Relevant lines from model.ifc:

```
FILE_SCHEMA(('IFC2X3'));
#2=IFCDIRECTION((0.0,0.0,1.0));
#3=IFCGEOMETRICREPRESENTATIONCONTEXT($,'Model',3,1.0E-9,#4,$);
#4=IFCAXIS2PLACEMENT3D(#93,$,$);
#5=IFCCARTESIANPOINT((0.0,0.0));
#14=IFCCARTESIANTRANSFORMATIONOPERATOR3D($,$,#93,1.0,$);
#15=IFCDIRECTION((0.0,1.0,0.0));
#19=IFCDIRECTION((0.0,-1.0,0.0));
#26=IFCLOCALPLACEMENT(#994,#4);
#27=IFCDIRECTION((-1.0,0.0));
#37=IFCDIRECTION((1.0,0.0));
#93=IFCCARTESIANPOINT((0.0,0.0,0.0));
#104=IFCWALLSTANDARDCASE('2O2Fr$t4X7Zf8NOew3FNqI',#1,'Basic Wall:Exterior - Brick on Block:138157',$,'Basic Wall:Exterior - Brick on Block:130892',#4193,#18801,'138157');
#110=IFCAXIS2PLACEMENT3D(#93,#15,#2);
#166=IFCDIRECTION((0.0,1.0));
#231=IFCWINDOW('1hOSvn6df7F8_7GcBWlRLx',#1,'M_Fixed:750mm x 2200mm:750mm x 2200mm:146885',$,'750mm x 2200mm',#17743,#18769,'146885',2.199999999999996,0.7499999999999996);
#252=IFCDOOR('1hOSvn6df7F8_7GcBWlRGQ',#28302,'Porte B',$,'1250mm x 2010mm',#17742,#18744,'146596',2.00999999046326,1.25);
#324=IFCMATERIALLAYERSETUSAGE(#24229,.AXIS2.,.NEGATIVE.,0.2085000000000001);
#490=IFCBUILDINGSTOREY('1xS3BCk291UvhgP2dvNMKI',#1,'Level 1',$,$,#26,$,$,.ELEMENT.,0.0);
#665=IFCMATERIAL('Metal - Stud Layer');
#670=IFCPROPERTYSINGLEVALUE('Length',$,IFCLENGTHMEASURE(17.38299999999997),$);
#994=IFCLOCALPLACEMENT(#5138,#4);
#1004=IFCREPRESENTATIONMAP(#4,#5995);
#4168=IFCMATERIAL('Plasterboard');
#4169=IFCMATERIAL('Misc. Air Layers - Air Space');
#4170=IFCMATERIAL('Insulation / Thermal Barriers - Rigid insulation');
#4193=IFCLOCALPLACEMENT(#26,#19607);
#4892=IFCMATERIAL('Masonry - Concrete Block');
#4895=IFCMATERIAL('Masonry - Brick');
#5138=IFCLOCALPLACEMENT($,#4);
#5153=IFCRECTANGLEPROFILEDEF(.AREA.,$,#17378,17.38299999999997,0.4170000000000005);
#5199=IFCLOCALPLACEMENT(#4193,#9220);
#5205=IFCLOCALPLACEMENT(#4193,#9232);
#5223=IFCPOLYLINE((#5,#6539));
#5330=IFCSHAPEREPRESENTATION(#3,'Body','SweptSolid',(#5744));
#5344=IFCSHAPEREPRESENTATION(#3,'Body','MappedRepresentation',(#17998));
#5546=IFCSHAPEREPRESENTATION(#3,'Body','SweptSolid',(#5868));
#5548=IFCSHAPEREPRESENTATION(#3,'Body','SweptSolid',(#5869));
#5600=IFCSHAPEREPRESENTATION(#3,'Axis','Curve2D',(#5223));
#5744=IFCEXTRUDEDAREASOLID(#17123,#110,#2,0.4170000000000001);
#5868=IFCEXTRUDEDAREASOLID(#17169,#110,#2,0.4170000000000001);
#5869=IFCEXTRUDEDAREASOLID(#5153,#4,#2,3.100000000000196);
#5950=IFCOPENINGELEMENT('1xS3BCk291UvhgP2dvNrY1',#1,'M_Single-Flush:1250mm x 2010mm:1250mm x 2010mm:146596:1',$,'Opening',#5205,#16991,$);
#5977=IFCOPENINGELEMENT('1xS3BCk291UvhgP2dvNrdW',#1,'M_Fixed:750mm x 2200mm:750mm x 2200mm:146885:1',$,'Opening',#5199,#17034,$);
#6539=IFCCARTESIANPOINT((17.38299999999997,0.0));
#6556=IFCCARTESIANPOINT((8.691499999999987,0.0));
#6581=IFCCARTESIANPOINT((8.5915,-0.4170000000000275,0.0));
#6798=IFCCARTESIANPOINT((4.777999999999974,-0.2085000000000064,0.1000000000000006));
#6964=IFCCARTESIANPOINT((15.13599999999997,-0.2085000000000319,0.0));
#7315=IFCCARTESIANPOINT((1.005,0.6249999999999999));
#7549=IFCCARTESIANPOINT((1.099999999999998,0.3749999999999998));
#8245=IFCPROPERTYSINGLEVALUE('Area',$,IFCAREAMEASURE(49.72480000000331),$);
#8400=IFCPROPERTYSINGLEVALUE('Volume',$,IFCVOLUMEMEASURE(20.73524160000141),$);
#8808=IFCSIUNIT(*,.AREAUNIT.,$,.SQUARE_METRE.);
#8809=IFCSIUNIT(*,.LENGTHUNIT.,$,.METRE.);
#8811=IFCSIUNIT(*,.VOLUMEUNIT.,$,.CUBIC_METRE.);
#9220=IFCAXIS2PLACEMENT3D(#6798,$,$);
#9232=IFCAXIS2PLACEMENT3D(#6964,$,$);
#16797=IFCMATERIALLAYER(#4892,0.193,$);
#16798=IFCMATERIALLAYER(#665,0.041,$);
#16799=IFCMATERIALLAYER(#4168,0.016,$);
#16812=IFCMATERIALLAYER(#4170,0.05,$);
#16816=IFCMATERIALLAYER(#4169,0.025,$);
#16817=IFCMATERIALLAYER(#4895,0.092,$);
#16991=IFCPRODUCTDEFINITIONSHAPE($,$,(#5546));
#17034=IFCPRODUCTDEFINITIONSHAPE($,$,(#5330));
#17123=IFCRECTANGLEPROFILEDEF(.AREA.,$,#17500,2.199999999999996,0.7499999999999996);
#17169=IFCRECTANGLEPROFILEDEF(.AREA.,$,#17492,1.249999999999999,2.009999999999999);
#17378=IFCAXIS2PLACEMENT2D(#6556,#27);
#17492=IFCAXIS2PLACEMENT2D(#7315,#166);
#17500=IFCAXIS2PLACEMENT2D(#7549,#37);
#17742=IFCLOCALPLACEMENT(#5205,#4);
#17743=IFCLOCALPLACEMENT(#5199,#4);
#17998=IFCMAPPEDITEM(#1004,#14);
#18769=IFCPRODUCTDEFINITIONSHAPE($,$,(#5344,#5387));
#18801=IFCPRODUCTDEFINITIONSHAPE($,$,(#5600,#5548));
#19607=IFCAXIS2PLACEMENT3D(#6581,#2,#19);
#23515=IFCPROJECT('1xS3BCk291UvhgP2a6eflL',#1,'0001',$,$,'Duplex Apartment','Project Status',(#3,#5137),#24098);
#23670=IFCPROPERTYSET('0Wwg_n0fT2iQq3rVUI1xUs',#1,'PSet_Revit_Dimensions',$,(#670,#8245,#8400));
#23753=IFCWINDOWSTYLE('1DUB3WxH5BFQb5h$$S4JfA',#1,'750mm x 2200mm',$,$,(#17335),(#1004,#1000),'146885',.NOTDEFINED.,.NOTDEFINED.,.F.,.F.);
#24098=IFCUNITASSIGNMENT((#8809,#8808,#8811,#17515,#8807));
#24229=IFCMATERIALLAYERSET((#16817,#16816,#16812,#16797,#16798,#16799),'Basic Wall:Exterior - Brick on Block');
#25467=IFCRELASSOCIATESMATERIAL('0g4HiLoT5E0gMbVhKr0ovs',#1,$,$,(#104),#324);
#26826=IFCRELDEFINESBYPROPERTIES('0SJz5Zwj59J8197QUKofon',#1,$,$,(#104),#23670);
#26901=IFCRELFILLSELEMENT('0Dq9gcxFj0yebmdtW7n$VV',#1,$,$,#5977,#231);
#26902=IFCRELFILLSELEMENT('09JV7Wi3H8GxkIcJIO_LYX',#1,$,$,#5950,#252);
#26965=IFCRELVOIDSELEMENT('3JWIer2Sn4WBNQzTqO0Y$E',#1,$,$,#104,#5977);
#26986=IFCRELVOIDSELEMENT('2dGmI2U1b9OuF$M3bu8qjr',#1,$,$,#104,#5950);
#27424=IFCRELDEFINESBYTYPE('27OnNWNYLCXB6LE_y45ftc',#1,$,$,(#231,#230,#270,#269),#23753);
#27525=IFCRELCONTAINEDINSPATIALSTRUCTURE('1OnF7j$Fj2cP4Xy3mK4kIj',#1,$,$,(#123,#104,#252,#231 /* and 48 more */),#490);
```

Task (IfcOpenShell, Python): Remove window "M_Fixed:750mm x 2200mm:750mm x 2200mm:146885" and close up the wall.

```python
import ifcopenshell
import ifcopenshell.api.feature
import ifcopenshell.api.pset
import ifcopenshell.api.root
import ifcopenshell.geom
import ifcopenshell.util.element
import ifcopenshell.util.shape
import ifcopenshell.util.unit

model = ifcopenshell.open("model.ifc")
area_scale = ifcopenshell.util.unit.calculate_unit_scale(model, "AREAUNIT")
volume_scale = ifcopenshell.util.unit.calculate_unit_scale(model, "VOLUMEUNIT")
settings = ifcopenshell.geom.settings()


def volume(element):
    """Net volume in cubic metres, openings subtracted."""
    shape = ifcopenshell.geom.create_shape(settings, element)
    return ifcopenshell.util.shape.get_volume(shape.geometry)


window = model.by_id(231)
opening = window.FillsVoids[0].RelatingOpeningElement
wall = opening.VoidsElements[0].RelatingBuildingElement
before = volume(wall)

ifcopenshell.api.root.remove_product(model, product=window)
ifcopenshell.api.feature.remove_feature(model, feature=opening)

after = volume(wall)
thickness = 0.417  # wall thickness in metres

# Update the wall's stored quantities.
pset = model.by_id(ifcopenshell.util.element.get_pset(wall, "PSet_Revit_Dimensions", should_inherit=False)["id"])
ifcopenshell.api.pset.edit_pset(model, pset=pset, properties={
    "Area": model.create_entity("IfcAreaMeasure", after / thickness / area_scale),
    "Volume": model.create_entity("IfcVolumeMeasure", after / volume_scale),
})

print(f"wall volume {before:.3f} -> {after:.3f} m3")

model.write("model_edited.ifc")
```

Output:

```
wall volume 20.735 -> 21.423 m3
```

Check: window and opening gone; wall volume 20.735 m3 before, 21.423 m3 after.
